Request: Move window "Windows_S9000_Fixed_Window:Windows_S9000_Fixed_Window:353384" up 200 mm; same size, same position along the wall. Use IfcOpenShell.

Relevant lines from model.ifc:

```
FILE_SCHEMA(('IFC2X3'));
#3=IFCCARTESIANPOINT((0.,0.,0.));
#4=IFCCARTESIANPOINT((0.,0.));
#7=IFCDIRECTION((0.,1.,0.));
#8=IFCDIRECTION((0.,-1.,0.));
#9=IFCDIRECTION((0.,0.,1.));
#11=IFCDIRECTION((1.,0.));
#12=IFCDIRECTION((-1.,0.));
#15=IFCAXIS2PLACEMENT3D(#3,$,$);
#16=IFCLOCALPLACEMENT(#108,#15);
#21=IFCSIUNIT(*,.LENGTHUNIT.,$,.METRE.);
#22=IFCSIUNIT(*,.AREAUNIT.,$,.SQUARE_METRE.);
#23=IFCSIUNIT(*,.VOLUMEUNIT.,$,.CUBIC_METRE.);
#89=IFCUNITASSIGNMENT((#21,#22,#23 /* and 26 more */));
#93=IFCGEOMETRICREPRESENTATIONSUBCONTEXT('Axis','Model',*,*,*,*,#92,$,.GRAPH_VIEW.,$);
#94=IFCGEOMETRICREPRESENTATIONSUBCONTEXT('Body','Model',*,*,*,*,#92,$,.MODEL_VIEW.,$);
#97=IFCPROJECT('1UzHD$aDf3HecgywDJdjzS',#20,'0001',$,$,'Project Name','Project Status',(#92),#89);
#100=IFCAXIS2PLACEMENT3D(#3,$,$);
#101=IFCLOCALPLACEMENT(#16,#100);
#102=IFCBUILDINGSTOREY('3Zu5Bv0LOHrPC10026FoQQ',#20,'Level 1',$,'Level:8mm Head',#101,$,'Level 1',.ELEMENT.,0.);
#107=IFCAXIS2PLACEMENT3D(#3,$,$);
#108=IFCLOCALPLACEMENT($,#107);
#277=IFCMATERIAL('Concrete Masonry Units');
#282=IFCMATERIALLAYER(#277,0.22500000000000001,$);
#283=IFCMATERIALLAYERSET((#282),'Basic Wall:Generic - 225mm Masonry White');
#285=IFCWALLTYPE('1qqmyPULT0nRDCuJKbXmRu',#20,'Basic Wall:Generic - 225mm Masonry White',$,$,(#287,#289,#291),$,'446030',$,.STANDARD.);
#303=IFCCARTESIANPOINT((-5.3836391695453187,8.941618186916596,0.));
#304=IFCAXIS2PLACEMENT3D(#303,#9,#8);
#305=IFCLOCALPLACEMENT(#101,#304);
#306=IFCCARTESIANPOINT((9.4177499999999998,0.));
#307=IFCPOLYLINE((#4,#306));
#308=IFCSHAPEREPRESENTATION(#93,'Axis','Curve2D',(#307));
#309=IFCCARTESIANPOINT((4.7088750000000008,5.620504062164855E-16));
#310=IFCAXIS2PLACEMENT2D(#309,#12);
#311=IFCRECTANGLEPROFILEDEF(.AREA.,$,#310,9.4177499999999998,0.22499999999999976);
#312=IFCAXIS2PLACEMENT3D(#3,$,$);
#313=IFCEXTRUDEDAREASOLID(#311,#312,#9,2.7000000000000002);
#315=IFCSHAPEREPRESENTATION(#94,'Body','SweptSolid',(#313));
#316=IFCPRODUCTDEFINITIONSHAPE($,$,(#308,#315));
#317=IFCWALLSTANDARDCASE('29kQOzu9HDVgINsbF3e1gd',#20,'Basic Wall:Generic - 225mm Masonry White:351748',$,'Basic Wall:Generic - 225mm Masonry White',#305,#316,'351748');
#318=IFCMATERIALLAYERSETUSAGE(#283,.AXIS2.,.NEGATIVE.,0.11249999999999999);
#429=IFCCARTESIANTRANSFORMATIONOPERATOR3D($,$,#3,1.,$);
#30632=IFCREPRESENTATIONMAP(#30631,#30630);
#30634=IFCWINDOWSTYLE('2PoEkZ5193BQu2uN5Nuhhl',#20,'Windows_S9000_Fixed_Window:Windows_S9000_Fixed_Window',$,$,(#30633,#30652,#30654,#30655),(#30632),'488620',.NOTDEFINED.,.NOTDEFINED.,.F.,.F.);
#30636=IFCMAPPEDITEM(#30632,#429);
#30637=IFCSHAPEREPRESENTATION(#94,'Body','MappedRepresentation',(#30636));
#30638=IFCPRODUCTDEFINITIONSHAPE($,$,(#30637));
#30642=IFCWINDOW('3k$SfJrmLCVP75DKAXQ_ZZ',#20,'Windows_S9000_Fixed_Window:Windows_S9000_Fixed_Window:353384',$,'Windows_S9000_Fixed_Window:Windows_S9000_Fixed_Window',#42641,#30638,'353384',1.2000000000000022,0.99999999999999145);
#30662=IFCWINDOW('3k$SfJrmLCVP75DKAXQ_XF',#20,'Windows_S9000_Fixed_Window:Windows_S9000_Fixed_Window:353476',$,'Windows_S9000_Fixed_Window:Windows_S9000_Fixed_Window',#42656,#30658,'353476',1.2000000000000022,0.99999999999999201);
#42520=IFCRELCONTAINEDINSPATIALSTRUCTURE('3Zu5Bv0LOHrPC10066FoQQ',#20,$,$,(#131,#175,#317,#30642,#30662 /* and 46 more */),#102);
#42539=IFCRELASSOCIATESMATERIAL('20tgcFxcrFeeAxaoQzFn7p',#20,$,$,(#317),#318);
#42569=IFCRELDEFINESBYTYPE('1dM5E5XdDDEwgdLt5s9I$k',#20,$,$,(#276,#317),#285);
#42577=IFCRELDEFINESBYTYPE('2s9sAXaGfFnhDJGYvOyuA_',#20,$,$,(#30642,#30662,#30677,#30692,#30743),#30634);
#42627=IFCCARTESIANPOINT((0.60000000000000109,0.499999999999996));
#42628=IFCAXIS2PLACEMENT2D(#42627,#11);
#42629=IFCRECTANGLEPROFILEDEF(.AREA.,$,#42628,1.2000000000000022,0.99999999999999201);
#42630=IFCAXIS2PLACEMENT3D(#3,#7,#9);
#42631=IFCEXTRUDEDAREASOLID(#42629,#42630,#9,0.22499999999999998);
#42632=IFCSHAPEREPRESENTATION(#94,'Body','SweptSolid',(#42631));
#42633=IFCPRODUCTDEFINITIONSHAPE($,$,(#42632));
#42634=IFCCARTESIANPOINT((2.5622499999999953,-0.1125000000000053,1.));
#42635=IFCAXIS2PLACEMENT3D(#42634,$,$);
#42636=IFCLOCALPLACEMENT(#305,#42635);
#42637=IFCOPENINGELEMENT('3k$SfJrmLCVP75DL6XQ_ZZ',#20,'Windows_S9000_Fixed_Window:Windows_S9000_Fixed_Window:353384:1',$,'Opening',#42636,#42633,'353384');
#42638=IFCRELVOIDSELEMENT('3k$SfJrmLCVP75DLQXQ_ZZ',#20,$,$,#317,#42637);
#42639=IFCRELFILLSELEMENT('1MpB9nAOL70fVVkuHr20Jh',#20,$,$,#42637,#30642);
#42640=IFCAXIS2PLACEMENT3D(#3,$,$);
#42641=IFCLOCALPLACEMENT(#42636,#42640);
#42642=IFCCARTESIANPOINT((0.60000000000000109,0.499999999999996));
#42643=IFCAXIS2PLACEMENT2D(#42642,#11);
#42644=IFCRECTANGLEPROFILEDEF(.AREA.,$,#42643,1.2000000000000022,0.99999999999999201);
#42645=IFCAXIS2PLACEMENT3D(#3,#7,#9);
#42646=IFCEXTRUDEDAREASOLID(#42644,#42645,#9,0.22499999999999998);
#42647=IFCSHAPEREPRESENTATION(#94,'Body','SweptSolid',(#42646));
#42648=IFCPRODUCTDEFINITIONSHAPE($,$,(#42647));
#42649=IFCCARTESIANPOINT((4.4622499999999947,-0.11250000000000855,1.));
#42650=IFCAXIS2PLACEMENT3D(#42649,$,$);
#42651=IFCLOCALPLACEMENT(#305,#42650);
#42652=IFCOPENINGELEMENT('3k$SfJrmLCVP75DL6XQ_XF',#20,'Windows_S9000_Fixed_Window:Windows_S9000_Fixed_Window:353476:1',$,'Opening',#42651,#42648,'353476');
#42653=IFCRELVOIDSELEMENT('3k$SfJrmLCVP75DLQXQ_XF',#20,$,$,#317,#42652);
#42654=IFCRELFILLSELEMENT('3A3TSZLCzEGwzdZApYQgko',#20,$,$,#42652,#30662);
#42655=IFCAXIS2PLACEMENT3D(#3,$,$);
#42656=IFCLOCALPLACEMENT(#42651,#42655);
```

```python
import numpy as np
import ifcopenshell
import ifcopenshell.api.geometry
import ifcopenshell.util.placement
import ifcopenshell.util.unit

model = ifcopenshell.open("model.ifc")
unit_scale = ifcopenshell.util.unit.calculate_unit_scale(model)

window = model.by_guid("3k$SfJrmLCVP75DKAXQ_ZZ")
opening = window.FillsVoids[0].RelatingOpeningElement
dz = 0.2 / unit_scale

shift = np.array([0.0, 0.0, dz])
# The window is placed relative to its opening, so it follows when the opening moves.
matrix = ifcopenshell.util.placement.get_local_placement(opening.ObjectPlacement)
matrix[:3, 3] += shift
ifcopenshell.api.geometry.edit_object_placement(
    model, product=opening, matrix=matrix, is_si=False, should_transform_children=True
)

print(f"moved by {dz * unit_scale:+.3f} m")

model.write("model_v2.ifc")
```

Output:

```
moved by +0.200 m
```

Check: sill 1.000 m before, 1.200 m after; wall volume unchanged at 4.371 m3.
